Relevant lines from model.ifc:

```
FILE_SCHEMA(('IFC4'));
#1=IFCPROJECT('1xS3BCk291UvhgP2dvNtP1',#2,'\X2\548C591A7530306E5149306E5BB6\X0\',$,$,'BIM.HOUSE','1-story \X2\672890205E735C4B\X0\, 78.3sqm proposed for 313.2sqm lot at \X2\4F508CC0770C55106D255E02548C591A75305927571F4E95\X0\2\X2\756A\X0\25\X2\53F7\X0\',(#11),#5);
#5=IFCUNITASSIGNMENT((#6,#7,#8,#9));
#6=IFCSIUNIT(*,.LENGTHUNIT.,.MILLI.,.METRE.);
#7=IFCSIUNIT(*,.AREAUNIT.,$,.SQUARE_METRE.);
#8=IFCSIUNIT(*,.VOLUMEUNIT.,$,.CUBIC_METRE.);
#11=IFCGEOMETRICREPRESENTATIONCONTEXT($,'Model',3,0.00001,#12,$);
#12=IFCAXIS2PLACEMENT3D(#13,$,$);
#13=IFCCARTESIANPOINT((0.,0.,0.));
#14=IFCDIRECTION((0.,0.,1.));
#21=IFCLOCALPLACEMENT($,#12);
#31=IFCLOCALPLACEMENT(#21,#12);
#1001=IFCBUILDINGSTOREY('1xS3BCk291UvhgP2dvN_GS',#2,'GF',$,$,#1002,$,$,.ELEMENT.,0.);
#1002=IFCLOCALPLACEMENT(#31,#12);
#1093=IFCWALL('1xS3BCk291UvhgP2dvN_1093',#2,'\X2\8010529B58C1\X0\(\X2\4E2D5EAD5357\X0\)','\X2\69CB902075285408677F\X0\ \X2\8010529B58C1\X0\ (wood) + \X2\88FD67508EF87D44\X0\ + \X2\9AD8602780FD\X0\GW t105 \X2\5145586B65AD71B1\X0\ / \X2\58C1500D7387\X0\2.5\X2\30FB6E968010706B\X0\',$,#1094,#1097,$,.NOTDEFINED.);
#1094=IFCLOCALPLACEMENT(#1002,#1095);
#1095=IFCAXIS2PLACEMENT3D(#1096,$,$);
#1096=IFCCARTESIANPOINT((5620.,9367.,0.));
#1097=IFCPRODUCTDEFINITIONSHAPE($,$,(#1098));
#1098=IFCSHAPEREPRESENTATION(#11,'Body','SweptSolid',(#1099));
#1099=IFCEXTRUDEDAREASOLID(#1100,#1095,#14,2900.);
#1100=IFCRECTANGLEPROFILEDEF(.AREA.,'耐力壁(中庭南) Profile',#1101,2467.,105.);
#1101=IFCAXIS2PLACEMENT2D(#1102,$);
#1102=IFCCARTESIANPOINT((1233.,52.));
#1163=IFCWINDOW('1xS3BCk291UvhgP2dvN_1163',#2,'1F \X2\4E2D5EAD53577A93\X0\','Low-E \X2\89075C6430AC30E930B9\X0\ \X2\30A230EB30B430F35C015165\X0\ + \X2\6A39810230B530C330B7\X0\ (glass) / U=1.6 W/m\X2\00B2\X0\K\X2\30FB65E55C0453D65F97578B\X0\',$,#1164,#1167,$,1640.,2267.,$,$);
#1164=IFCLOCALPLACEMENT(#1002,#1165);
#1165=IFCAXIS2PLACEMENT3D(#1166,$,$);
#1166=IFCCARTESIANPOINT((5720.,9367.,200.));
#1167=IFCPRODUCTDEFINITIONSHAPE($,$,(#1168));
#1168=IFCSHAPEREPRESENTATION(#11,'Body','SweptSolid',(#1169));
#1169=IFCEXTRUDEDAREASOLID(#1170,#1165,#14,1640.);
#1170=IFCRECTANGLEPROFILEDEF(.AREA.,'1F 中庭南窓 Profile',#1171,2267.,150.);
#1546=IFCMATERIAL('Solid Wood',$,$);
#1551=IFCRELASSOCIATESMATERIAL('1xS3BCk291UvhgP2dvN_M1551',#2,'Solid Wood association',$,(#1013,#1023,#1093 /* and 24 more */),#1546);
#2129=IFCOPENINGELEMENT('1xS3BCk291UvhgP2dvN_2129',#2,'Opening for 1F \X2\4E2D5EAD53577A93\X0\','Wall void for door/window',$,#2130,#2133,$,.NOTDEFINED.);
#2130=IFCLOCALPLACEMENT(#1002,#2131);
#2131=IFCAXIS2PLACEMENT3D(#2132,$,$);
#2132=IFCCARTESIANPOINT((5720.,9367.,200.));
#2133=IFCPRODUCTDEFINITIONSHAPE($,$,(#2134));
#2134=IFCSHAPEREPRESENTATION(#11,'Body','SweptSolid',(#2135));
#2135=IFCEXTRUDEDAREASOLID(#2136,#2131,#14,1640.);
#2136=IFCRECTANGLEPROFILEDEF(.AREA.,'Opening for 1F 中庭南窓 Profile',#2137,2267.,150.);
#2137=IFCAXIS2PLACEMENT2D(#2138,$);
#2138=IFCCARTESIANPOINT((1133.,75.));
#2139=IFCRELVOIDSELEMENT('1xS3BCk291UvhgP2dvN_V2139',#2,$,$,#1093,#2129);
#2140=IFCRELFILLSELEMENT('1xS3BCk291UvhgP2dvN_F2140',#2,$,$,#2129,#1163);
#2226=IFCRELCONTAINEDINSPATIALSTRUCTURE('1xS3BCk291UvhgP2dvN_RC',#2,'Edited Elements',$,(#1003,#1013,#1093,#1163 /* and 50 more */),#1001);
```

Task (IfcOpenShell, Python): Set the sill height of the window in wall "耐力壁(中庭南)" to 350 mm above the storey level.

```python
import numpy as np
import ifcopenshell
import ifcopenshell.api.geometry
import ifcopenshell.geom
import ifcopenshell.util.element
import ifcopenshell.util.placement
import ifcopenshell.util.shape
import ifcopenshell.util.unit

model = ifcopenshell.open("model.ifc")
unit_scale = ifcopenshell.util.unit.calculate_unit_scale(model)

window = model.by_id(1163)
opening = window.FillsVoids[0].RelatingOpeningElement
storey = ifcopenshell.util.element.get_container(window, ifc_class="IfcBuildingStorey")
level = ifcopenshell.util.placement.get_local_placement(storey.ObjectPlacement)[2, 3]

# The opening's origin need not be at the sill, so measure its lowest point.
shape = ifcopenshell.geom.create_shape(ifcopenshell.geom.settings(), opening)
bottom = ifcopenshell.util.shape.get_shape_bottom_elevation(shape, shape.geometry) / unit_scale
dz = level + 350.0 - bottom

shift = np.array([0.0, 0.0, dz])
# The window is not placed relative to its opening, so move both.
for product in (opening, window):
    matrix = ifcopenshell.util.placement.get_local_placement(product.ObjectPlacement)
    matrix[:3, 3] += shift
    ifcopenshell.api.geometry.edit_object_placement(model, product=product, matrix=matrix, is_si=False)

print(f"moved by {dz * unit_scale:+.3f} m")

model.write("model-out.ifc")
```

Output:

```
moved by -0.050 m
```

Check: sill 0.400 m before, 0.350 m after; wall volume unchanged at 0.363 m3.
